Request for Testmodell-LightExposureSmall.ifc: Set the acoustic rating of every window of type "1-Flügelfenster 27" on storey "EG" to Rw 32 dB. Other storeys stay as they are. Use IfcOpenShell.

First a look at what the model holds.

```python
import ifcopenshell
import ifcopenshell.util.element

model = ifcopenshell.open("Testmodell-LightExposureSmall.ifc")
print(model.schema)
storey = next(s for s in model.by_type("IfcBuildingStorey") if s.Name == "EG")
windows = [e for e in ifcopenshell.util.element.get_decomposition(storey) if e.is_a("IfcWindow")]
seen = {}
for e in windows:
    element_type = ifcopenshell.util.element.get_type(e)
    key = (element_type.Name if element_type != e and element_type else None, ifcopenshell.util.element.get_pset(e, "Pset_WindowCommon", "AcousticRating"))
    seen[key] = seen.get(key, 0) + 1
for (name, value), count in sorted(seen.items(), key=str):
    print(count, "x", name, "|", value)
```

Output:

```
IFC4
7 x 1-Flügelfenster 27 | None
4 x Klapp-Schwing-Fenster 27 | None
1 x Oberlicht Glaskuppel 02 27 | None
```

```python
import ifcopenshell
import ifcopenshell.api.pset
import ifcopenshell.util.element

model = ifcopenshell.open("Testmodell-LightExposureSmall.ifc")

storey = next(s for s in model.by_type("IfcBuildingStorey") if s.Name == "EG")
windows = [e for e in ifcopenshell.util.element.get_decomposition(storey) if e.is_a("IfcWindow")]

count = 0
for e in windows:
    element_type = ifcopenshell.util.element.get_type(e)
    if element_type in (None, e) or element_type.Name != "1-Flügelfenster 27":
        continue
    # add_pset returns the element's existing set when there is one.
    pset = ifcopenshell.api.pset.add_pset(model, product=e, name="Pset_WindowCommon")
    ifcopenshell.api.pset.edit_pset(model, pset=pset, properties={"AcousticRating": "Rw 32 dB"})
    count += 1

print(count, "windows updated")

model.write("Testmodell-LightExposureSmall_updated.ifc")
```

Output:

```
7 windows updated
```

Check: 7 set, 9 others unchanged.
